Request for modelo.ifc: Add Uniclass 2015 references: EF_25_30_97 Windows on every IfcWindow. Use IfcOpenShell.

First a look at what the model holds.

```python
import ifcopenshell

model = ifcopenshell.open("modelo.ifc")
print(model.schema)
print("classifications:", [c.Name for c in model.by_type("IfcClassification")])
for ifc_class in ("IfcDoor", "IfcRoof", "IfcStair", "IfcWall", "IfcWindow"):
    print(ifc_class, len(model.by_type(ifc_class)))
```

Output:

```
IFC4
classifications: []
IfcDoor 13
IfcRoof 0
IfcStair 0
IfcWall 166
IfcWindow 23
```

```python
import ifcopenshell
import ifcopenshell.api.classification

model = ifcopenshell.open("modelo.ifc")

system = ifcopenshell.api.classification.add_classification(model, classification="Uniclass 2015")

codes = {
    "IfcWindow": ("EF_25_30_97", "Windows"),
}
for ifc_class, (code, name) in codes.items():
    products = model.by_type(ifc_class)
    ifcopenshell.api.classification.add_reference(
        model, products=products, classification=system, identification=code, name=name
    )
    print(code, len(products))

model.write("modelo_rev.ifc")
```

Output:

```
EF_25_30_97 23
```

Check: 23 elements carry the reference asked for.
